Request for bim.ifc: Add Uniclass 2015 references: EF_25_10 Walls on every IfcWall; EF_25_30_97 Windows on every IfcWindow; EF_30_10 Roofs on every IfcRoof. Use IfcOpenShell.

First a look at what the model holds.

```python
import ifcopenshell

model = ifcopenshell.open("bim.ifc")
print(model.schema)
print("classifications:", [c.Name for c in model.by_type("IfcClassification")])
for ifc_class in ("IfcDoor", "IfcRoof", "IfcStair", "IfcWall", "IfcWindow"):
    print(ifc_class, len(model.by_type(ifc_class)))
```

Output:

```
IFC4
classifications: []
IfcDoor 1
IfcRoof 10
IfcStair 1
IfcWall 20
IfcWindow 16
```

```python
import ifcopenshell
import ifcopenshell.api.classification

model = ifcopenshell.open("bim.ifc")

system = ifcopenshell.api.classification.add_classification(model, classification="Uniclass 2015")

codes = {
    "IfcWall": ("EF_25_10", "Walls"),
    "IfcWindow": ("EF_25_30_97", "Windows"),
    "IfcRoof": ("EF_30_10", "Roofs"),
}
for ifc_class, (code, name) in codes.items():
    products = model.by_type(ifc_class)
    ifcopenshell.api.classification.add_reference(
        model, products=products, classification=system, identification=code, name=name
    )
    print(code, len(products))

model.write("bim_rev.ifc")
```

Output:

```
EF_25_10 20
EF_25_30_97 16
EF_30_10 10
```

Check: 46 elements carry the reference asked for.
